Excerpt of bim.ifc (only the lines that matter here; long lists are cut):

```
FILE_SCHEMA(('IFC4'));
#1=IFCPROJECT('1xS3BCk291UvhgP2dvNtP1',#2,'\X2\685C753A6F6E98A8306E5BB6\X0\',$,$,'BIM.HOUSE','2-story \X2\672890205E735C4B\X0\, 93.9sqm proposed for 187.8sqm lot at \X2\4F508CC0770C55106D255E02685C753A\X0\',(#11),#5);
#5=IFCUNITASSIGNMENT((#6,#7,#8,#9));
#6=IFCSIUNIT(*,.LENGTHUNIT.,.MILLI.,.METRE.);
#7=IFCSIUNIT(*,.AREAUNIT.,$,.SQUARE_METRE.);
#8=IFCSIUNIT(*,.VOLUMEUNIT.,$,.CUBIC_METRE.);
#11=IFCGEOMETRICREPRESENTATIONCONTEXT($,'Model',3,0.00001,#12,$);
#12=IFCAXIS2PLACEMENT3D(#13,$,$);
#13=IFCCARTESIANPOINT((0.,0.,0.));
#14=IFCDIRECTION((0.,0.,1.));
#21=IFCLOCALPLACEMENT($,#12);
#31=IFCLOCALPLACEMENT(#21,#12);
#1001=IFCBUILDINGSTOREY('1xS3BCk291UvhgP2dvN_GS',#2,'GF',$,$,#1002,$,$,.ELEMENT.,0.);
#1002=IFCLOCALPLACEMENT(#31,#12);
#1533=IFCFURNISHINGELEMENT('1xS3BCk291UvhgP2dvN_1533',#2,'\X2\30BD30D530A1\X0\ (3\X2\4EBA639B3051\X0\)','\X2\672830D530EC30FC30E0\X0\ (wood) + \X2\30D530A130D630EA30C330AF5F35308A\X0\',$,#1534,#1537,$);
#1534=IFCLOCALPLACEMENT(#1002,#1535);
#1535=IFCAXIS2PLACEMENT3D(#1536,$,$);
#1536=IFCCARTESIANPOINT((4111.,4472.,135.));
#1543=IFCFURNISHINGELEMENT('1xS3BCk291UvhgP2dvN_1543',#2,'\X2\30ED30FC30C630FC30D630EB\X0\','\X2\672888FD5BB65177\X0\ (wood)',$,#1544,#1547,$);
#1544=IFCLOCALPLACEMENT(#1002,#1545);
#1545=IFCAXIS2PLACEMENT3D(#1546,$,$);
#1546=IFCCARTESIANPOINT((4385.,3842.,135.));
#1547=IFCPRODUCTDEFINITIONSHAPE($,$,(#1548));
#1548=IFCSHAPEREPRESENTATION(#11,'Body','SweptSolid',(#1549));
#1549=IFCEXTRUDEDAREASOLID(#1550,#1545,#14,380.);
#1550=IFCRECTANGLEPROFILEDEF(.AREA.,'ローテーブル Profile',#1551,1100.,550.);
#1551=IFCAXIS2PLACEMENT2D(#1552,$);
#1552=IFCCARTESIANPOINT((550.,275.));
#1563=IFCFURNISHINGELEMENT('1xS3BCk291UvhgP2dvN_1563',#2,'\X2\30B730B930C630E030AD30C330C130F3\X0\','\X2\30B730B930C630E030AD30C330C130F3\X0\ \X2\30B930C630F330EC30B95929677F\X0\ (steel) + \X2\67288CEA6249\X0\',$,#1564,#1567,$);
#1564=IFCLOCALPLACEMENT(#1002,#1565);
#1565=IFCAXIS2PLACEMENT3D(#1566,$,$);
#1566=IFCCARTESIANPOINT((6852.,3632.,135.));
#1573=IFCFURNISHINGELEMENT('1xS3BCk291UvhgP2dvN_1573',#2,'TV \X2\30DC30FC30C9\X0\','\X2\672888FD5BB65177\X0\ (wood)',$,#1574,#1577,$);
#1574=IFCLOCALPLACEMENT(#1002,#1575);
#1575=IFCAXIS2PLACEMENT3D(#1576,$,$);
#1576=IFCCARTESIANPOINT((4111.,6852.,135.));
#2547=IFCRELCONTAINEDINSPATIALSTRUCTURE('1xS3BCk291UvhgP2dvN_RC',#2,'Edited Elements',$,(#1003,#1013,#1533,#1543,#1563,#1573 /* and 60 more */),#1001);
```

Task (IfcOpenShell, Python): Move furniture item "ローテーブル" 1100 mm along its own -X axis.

```python
import ifcopenshell
import ifcopenshell.api.geometry
import ifcopenshell.util.placement

model = ifcopenshell.open("bim.ifc")

item = model.by_id(1543)
matrix = ifcopenshell.util.placement.get_local_placement(item.ObjectPlacement)
matrix[:3, 3] -= matrix[:3, 0] * 1100.0
ifcopenshell.api.geometry.edit_object_placement(model, product=item, matrix=matrix, is_si=False)

print(ifcopenshell.util.placement.get_local_placement(item.ObjectPlacement).round(3) + 0.0)

model.write("bim_v2.ifc")
```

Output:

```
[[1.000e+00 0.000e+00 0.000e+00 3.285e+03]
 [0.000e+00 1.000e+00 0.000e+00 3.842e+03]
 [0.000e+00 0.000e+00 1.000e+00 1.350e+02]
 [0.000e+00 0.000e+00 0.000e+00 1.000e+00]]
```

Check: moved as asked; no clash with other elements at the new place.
